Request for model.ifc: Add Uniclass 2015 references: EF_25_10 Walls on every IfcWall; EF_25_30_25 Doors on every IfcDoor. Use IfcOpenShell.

First a look at what the model holds.

```python
import ifcopenshell

model = ifcopenshell.open("model.ifc")
print(model.schema)
print("classifications:", [c.Name for c in model.by_type("IfcClassification")])
for ifc_class in ("IfcDoor", "IfcRoof", "IfcStair", "IfcWall", "IfcWindow"):
    print(ifc_class, len(model.by_type(ifc_class)))
```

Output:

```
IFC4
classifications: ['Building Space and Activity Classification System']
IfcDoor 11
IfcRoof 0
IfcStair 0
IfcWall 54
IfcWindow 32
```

```python
import ifcopenshell
import ifcopenshell.api.classification

model = ifcopenshell.open("model.ifc")

system = ifcopenshell.api.classification.add_classification(model, classification="Uniclass 2015")

codes = {
    "IfcWall": ("EF_25_10", "Walls"),
    "IfcDoor": ("EF_25_30_25", "Doors"),
}
for ifc_class, (code, name) in codes.items():
    products = model.by_type(ifc_class)
    ifcopenshell.api.classification.add_reference(
        model, products=products, classification=system, identification=code, name=name
    )
    print(code, len(products))

model.write("model-out.ifc")
```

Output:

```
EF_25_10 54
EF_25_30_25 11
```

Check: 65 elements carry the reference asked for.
